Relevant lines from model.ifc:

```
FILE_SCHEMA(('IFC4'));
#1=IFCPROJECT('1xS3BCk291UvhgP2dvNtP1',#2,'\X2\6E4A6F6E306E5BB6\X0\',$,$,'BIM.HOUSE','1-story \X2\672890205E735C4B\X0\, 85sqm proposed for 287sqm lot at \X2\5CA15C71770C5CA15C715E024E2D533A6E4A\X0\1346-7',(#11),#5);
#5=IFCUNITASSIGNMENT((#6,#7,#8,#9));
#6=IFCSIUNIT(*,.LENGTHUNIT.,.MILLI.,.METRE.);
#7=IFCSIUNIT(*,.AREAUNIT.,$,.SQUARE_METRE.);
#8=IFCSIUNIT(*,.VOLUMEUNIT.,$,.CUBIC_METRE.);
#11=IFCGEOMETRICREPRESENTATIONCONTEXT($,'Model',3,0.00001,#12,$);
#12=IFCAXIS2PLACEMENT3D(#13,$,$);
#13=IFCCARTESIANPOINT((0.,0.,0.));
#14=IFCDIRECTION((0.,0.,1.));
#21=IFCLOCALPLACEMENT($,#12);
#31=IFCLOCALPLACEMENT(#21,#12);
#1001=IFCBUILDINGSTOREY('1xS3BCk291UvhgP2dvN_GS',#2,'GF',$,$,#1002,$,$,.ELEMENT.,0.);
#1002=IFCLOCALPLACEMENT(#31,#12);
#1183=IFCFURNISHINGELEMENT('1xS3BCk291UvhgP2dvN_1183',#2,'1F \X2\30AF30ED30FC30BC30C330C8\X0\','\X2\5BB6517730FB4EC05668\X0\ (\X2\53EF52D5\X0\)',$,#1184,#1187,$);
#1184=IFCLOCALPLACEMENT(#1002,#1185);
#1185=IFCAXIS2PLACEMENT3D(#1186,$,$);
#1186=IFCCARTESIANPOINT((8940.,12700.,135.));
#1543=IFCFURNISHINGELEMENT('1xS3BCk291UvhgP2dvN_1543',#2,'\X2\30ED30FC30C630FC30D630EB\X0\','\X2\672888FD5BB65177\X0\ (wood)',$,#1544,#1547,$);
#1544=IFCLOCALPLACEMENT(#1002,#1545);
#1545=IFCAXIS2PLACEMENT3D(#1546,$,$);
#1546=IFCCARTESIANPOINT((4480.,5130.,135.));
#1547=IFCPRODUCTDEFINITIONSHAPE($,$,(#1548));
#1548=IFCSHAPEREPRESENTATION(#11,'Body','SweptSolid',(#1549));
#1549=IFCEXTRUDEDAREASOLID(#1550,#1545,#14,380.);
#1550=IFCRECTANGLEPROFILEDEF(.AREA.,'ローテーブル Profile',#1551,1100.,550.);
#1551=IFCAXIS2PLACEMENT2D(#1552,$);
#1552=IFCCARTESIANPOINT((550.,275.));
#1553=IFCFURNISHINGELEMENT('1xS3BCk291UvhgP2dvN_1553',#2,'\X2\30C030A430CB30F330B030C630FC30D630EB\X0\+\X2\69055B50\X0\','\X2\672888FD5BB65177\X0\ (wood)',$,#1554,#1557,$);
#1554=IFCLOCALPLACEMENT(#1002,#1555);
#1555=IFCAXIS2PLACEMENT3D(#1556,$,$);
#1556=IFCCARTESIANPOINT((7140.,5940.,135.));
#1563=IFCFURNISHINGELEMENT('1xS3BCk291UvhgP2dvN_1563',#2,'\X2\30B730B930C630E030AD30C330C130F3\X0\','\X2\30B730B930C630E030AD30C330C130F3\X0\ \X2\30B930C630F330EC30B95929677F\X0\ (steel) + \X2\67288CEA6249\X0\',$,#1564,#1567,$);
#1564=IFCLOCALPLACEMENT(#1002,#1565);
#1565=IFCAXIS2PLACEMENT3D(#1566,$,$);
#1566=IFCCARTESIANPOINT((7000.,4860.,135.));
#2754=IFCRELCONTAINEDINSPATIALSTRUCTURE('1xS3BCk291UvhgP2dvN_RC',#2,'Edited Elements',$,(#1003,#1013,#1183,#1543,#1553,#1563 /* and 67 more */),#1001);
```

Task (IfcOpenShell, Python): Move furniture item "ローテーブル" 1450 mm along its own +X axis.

```python
import ifcopenshell
import ifcopenshell.api.geometry
import ifcopenshell.util.placement
import ifcopenshell.util.unit

model = ifcopenshell.open("model.ifc")
unit_scale = ifcopenshell.util.unit.calculate_unit_scale(model)

item = model.by_guid("1xS3BCk291UvhgP2dvN_1543")
matrix = ifcopenshell.util.placement.get_local_placement(item.ObjectPlacement)
matrix[:3, 3] += matrix[:3, 0] * 1.45 / unit_scale
ifcopenshell.api.geometry.edit_object_placement(model, product=item, matrix=matrix, is_si=False)

print(ifcopenshell.util.placement.get_local_placement(item.ObjectPlacement).round(3) + 0.0)

model.write("model_v2.ifc")
```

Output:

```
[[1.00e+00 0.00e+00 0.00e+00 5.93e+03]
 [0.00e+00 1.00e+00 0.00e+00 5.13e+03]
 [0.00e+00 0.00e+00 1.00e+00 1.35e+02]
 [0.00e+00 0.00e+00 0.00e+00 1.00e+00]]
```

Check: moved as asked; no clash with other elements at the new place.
